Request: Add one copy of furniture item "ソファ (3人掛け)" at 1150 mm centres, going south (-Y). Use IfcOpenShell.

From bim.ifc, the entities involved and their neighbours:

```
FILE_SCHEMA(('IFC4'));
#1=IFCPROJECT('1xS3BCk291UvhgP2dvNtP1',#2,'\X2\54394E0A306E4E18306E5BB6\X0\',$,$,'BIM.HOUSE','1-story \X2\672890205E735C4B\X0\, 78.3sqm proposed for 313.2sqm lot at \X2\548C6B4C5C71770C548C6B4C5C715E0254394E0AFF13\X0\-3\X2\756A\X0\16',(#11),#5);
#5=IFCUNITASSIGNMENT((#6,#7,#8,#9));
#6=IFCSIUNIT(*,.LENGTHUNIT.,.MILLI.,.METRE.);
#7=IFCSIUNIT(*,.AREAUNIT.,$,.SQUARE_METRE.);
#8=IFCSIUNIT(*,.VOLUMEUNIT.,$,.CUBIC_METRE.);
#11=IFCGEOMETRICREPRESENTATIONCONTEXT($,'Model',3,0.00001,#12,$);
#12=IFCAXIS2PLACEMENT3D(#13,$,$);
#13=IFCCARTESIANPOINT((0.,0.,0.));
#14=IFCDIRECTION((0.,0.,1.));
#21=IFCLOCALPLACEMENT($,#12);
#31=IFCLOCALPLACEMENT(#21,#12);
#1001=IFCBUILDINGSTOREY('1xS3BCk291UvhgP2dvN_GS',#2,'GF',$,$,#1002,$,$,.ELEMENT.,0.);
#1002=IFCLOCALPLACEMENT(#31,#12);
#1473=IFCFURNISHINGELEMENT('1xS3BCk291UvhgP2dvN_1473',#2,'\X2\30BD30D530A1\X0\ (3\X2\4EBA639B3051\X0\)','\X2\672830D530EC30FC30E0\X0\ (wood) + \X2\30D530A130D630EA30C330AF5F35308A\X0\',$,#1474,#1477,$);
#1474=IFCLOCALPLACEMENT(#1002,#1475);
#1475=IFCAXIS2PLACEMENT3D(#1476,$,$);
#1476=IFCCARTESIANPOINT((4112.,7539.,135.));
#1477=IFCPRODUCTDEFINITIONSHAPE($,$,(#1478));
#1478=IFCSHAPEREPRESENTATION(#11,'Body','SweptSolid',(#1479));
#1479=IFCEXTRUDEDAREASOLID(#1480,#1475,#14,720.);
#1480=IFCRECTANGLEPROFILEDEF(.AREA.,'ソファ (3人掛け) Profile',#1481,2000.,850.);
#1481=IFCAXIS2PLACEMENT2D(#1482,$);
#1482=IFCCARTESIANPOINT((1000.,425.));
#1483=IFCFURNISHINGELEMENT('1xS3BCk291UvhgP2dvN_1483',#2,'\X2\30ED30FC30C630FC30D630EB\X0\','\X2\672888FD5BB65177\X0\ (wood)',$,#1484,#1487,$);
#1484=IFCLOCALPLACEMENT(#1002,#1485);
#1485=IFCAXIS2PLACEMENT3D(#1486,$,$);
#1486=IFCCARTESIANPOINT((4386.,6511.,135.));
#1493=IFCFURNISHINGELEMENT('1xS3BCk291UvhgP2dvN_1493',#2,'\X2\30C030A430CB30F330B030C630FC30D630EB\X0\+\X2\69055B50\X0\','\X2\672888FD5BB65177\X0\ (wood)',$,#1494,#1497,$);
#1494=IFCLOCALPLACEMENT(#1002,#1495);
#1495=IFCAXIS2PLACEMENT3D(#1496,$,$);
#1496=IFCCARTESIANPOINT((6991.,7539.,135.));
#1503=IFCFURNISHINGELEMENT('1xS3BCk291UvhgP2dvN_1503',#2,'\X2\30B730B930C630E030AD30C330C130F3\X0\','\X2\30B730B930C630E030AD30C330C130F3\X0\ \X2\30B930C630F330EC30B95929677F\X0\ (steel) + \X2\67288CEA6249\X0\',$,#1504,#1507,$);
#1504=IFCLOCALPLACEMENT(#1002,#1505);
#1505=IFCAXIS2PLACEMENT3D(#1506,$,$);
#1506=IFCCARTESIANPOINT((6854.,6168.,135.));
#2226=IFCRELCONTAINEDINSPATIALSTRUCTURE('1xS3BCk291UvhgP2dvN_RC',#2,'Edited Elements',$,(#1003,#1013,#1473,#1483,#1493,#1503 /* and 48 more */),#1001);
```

```python
import numpy as np
import ifcopenshell
import ifcopenshell.api.geometry
import ifcopenshell.api.root
import ifcopenshell.util.element
import ifcopenshell.util.placement
import ifcopenshell.util.unit

model = ifcopenshell.open("bim.ifc")
unit_scale = ifcopenshell.util.unit.calculate_unit_scale(model)


def reuse_history(source, copy):
    """copy_class also copies each property set's owner history, people and application; keep the originals."""
    for rel in copy.IsDefinedBy:
        if rel.is_a("IfcRelDefinesByProperties") and (history := rel.RelatingPropertyDefinition.OwnerHistory):
            rel.RelatingPropertyDefinition.OwnerHistory = source.OwnerHistory
            ifcopenshell.util.element.remove_deep2(model, history)


source = model.by_id(1473)
base = ifcopenshell.util.placement.get_local_placement(source.ObjectPlacement)
step = np.array([0.0, -1.0, 0.0]) * 1.15 / unit_scale

for i in range(1, 2):
    copy = ifcopenshell.api.root.copy_class(model, product=source)
    copy.Representation = ifcopenshell.util.element.copy_deep(
        model, source.Representation, exclude=["IfcGeometricRepresentationContext", "IfcRepresentationMap"]
    )
    reuse_history(source, copy)
    matrix = base.copy()
    matrix[:3, 3] += i * step
    print("added at", matrix[:3, 3].round(3) + 0.0)
    ifcopenshell.api.geometry.edit_object_placement(model, product=copy, matrix=matrix, is_si=False)

model.write("bim_edited.ifc")
```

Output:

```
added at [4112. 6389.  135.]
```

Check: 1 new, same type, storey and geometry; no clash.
